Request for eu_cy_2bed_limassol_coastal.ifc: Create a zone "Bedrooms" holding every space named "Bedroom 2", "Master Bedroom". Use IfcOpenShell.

First a look at what the model holds.

```python
import ifcopenshell

model = ifcopenshell.open("eu_cy_2bed_limassol_coastal.ifc")
print(model.schema)
seen = {}
for space in model.by_type("IfcSpace"):
    seen[space.LongName] = seen.get(space.LongName, 0) + 1
for name, count in sorted(seen.items(), key=str):
    print(count, "x", name)
print("zones:", [z.Name for z in model.by_type("IfcZone")][:20])
```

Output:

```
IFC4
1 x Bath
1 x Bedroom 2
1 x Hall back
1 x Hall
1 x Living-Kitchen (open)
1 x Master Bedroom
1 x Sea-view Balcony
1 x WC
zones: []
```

```python
import ifcopenshell
import ifcopenshell.api.group
import ifcopenshell.api.root

model = ifcopenshell.open("eu_cy_2bed_limassol_coastal.ifc")

names = {"Bedroom 2", "Master Bedroom"}
spaces = [s for s in model.by_type("IfcSpace") if s.LongName in names]

zone = ifcopenshell.api.root.create_entity(model, ifc_class="IfcZone", name="Bedrooms")
ifcopenshell.api.group.assign_group(model, products=spaces, group=zone)
print(len(spaces), "spaces in", zone.Name)

model.write("eu_cy_2bed_limassol_coastal_edited.ifc")
```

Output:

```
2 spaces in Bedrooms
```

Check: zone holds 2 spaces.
